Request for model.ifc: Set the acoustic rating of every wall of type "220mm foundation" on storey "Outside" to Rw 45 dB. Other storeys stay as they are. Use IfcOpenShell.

First a look at what the model holds.

```python
import ifcopenshell
import ifcopenshell.util.element

model = ifcopenshell.open("model.ifc")
print(model.schema)
storey = next(s for s in model.by_type("IfcBuildingStorey") if s.Name == "Outside")
walls = [e for e in ifcopenshell.util.element.get_decomposition(storey) if e.is_a("IfcWall")]
seen = {}
for e in walls:
    element_type = ifcopenshell.util.element.get_type(e)
    key = (element_type.Name if element_type != e and element_type else None, ifcopenshell.util.element.get_pset(e, "Pset_WallCommon", "AcousticRating"))
    seen[key] = seen.get(key, 0) + 1
for (name, value), count in sorted(seen.items(), key=str):
    print(count, "x", name, "|", value)
```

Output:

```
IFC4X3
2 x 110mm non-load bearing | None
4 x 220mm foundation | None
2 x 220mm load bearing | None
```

```python
import ifcopenshell
import ifcopenshell.api.pset
import ifcopenshell.util.element

model = ifcopenshell.open("model.ifc")

storey = next(s for s in model.by_type("IfcBuildingStorey") if s.Name == "Outside")
walls = [e for e in ifcopenshell.util.element.get_decomposition(storey) if e.is_a("IfcWall")]

count = 0
for e in walls:
    element_type = ifcopenshell.util.element.get_type(e)
    if element_type in (None, e) or element_type.Name != "220mm foundation":
        continue
    # add_pset returns the element's existing set when there is one.
    pset = ifcopenshell.api.pset.add_pset(model, product=e, name="Pset_WallCommon")
    ifcopenshell.api.pset.edit_pset(model, pset=pset, properties={"AcousticRating": "Rw 45 dB"})
    count += 1

print(count, "walls updated")

model.write("model_edited.ifc")
```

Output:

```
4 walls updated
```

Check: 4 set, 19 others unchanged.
